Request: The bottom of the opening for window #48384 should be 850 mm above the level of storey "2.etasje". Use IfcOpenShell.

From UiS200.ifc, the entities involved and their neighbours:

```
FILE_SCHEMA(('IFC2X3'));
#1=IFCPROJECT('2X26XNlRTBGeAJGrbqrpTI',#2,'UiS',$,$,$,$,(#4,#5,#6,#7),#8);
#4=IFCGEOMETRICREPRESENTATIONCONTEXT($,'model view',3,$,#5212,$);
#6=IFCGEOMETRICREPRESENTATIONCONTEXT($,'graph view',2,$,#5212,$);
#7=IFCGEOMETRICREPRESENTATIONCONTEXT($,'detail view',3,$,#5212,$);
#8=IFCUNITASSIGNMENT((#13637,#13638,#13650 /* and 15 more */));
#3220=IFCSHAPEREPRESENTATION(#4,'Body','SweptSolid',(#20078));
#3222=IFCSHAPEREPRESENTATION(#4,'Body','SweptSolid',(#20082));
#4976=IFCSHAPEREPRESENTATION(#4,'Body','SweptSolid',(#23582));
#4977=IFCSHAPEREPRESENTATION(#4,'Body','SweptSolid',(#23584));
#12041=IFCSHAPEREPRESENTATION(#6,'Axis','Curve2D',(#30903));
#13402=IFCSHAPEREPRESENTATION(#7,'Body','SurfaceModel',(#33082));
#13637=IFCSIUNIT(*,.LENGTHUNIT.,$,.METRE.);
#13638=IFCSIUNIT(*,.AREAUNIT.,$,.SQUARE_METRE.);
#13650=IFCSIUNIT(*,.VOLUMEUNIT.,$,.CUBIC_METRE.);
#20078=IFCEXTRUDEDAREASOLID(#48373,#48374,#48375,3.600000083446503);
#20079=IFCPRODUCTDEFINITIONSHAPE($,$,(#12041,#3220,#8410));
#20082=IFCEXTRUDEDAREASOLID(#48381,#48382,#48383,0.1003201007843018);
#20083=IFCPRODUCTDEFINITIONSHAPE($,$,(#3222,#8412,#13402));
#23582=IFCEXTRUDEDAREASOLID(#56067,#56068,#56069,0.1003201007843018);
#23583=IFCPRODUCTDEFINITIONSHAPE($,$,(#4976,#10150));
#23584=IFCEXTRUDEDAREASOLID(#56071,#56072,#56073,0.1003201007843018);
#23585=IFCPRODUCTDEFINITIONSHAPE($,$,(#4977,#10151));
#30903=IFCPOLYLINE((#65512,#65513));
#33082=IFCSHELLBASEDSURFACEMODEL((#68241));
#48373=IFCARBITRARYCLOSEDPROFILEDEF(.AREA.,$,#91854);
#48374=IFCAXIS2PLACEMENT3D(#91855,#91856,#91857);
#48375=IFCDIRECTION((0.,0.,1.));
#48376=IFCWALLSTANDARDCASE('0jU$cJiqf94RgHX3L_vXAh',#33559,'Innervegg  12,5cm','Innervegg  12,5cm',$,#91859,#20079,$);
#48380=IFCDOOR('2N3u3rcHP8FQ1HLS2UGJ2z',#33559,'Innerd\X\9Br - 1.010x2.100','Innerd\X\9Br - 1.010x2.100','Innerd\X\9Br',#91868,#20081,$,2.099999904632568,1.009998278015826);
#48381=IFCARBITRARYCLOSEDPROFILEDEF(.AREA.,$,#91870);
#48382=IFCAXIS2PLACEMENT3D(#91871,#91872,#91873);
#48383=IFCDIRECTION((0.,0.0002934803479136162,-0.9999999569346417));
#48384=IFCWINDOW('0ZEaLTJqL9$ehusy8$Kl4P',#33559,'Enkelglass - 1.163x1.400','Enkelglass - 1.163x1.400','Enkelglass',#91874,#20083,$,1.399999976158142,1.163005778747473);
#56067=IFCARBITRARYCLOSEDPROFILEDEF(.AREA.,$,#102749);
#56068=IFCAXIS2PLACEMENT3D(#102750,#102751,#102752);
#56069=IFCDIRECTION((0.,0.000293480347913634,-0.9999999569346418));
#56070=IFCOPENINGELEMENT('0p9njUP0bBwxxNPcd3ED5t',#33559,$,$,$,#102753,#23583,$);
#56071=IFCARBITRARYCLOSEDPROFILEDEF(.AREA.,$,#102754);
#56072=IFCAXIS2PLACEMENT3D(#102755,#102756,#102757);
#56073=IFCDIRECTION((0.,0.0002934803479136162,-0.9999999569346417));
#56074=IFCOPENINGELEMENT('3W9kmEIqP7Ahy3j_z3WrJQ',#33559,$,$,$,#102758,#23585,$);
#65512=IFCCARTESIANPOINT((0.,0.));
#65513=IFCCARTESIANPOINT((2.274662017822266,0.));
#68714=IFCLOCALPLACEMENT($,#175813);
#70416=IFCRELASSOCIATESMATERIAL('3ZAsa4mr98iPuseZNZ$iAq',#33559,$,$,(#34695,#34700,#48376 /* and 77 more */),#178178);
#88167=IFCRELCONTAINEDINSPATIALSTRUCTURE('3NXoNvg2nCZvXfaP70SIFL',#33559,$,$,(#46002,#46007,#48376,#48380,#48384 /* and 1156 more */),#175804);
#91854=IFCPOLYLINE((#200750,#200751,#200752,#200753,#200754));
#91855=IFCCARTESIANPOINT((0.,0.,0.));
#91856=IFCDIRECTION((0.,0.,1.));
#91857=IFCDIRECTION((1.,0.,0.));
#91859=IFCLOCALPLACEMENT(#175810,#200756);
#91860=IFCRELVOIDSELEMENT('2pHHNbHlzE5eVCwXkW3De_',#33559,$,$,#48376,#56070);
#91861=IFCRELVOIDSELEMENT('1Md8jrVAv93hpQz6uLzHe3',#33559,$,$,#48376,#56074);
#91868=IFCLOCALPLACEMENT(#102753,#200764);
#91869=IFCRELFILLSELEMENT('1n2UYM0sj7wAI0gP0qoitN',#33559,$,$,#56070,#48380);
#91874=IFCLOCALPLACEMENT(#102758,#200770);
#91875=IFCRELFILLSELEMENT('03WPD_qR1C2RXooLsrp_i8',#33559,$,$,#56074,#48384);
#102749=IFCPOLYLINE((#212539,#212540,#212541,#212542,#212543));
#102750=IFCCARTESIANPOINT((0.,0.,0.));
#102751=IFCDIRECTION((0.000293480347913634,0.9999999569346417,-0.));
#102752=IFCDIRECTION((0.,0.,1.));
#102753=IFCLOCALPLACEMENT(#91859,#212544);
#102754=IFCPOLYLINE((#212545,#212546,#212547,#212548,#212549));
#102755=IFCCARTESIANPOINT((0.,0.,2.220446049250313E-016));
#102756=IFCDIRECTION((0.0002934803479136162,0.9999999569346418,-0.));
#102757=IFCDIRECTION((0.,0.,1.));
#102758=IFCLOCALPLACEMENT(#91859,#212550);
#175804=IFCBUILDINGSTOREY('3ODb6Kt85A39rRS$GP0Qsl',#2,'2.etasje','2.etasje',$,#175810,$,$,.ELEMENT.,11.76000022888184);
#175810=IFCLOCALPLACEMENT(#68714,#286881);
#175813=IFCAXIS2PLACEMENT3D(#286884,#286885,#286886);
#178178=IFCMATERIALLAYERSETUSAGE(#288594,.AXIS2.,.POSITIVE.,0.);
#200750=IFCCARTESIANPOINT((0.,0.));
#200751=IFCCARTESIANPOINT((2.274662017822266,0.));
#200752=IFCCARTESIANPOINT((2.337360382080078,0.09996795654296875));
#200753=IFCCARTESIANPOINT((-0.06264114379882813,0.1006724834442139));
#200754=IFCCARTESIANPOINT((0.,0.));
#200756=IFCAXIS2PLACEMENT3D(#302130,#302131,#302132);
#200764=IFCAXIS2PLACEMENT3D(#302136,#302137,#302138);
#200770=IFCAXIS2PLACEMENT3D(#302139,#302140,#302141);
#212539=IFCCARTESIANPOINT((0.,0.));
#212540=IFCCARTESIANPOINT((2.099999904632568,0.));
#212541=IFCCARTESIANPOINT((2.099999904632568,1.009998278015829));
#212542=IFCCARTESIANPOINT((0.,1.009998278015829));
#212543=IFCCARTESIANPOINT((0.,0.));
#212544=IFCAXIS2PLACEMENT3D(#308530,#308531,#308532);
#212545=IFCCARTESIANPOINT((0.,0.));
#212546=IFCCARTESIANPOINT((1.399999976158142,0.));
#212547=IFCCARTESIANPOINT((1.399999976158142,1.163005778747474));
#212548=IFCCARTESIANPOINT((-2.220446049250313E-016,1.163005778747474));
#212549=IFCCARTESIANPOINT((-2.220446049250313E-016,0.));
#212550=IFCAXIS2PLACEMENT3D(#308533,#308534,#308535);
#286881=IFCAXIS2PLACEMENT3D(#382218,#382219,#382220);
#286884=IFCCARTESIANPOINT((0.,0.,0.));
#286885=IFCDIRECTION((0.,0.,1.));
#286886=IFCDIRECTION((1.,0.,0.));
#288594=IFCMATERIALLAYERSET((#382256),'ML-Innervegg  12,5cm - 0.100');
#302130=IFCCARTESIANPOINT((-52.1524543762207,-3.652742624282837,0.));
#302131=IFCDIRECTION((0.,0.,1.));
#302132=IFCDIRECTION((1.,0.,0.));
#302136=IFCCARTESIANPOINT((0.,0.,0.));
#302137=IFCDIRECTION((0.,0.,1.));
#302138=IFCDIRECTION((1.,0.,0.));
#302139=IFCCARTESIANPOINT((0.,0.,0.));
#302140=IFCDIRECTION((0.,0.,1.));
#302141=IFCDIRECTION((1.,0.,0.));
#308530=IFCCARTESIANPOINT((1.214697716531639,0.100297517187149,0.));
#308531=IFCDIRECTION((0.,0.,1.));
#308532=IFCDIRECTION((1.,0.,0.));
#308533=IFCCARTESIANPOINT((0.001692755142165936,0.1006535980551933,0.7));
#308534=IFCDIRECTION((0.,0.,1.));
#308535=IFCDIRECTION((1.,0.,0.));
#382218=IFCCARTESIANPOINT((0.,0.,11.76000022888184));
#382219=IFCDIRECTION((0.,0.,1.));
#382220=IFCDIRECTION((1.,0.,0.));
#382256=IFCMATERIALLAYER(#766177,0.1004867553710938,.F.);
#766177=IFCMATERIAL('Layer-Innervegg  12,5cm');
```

```python
import numpy as np
import ifcopenshell
import ifcopenshell.api.geometry
import ifcopenshell.geom
import ifcopenshell.util.element
import ifcopenshell.util.placement
import ifcopenshell.util.shape
import ifcopenshell.util.unit

model = ifcopenshell.open("UiS200.ifc")
unit_scale = ifcopenshell.util.unit.calculate_unit_scale(model)

window = model.by_guid("0ZEaLTJqL9$ehusy8$Kl4P")
opening = window.FillsVoids[0].RelatingOpeningElement
storey = ifcopenshell.util.element.get_container(window, ifc_class="IfcBuildingStorey")
level = ifcopenshell.util.placement.get_local_placement(storey.ObjectPlacement)[2, 3]

# The opening's origin need not be at the sill, so measure its lowest point.
shape = ifcopenshell.geom.create_shape(ifcopenshell.geom.settings(), opening)
bottom = ifcopenshell.util.shape.get_shape_bottom_elevation(shape, shape.geometry) / unit_scale
dz = level + 0.85 / unit_scale - bottom

shift = np.array([0.0, 0.0, dz])
# The window is placed relative to its opening, so it follows when the opening moves.
matrix = ifcopenshell.util.placement.get_local_placement(opening.ObjectPlacement)
matrix[:3, 3] += shift
ifcopenshell.api.geometry.edit_object_placement(
    model, product=opening, matrix=matrix, is_si=False, should_transform_children=True
)

print(f"moved by {dz * unit_scale:+.3f} m")

model.write("UiS200_updated.ifc")
```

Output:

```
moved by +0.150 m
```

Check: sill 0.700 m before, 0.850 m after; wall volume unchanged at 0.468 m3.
